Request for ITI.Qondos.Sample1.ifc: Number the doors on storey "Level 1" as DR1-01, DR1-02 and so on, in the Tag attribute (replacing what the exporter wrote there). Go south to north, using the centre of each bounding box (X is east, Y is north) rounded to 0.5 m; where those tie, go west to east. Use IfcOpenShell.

First a look at what the model holds.

```python
import ifcopenshell
import ifcopenshell.util.element
import ifcopenshell.util.placement

model = ifcopenshell.open("ITI.Qondos.Sample1.ifc")
print(model.schema)
storey = next(s for s in model.by_type("IfcBuildingStorey") if s.Name == "Level 1")
doors = [e for e in ifcopenshell.util.element.get_decomposition(storey) if e.is_a("IfcDoor")]
for e in sorted(doors, key=lambda e: e.id()):
    origin = ifcopenshell.util.placement.get_local_placement(e.ObjectPlacement)[:3, 3]
    print(e.id(), e.Tag, e.Name, origin.round(2) + 0.0, sep=" | ")
```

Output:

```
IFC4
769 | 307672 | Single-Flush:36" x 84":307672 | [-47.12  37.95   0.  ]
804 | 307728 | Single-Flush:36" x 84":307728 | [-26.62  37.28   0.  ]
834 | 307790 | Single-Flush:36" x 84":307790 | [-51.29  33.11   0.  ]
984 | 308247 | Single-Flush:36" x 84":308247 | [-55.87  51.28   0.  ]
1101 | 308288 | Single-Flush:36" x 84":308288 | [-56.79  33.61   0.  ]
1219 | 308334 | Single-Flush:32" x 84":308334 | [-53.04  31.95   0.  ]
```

```python
import ifcopenshell
import ifcopenshell.geom
import ifcopenshell.util.element
import ifcopenshell.util.shape

model = ifcopenshell.open("ITI.Qondos.Sample1.ifc")
settings = ifcopenshell.geom.settings()
settings.set("use-world-coords", True)


def centre(element):
    shape = ifcopenshell.geom.create_shape(settings, element)
    return ifcopenshell.util.shape.get_bbox_centroid(shape.geometry)


storey = next(s for s in model.by_type("IfcBuildingStorey") if s.Name == "Level 1")
doors = [e for e in ifcopenshell.util.element.get_decomposition(storey) if e.is_a("IfcDoor")]

# Insertion points can sit at a corner or the storey origin, so sort by the geometry (in metres).
centres = {e: centre(e) for e in doors}
doors.sort(key=lambda e: (round(centres[e][1] / 0.5), centres[e][0]))

for i, e in enumerate(doors, start=1):
    number = f"DR1-{i:02d}"
    e.Tag = number
    print(e.id(), number)

model.write("ITI.Qondos.Sample1_edited.ifc")
```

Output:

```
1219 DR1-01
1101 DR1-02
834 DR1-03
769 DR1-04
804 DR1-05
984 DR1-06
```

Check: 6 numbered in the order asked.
